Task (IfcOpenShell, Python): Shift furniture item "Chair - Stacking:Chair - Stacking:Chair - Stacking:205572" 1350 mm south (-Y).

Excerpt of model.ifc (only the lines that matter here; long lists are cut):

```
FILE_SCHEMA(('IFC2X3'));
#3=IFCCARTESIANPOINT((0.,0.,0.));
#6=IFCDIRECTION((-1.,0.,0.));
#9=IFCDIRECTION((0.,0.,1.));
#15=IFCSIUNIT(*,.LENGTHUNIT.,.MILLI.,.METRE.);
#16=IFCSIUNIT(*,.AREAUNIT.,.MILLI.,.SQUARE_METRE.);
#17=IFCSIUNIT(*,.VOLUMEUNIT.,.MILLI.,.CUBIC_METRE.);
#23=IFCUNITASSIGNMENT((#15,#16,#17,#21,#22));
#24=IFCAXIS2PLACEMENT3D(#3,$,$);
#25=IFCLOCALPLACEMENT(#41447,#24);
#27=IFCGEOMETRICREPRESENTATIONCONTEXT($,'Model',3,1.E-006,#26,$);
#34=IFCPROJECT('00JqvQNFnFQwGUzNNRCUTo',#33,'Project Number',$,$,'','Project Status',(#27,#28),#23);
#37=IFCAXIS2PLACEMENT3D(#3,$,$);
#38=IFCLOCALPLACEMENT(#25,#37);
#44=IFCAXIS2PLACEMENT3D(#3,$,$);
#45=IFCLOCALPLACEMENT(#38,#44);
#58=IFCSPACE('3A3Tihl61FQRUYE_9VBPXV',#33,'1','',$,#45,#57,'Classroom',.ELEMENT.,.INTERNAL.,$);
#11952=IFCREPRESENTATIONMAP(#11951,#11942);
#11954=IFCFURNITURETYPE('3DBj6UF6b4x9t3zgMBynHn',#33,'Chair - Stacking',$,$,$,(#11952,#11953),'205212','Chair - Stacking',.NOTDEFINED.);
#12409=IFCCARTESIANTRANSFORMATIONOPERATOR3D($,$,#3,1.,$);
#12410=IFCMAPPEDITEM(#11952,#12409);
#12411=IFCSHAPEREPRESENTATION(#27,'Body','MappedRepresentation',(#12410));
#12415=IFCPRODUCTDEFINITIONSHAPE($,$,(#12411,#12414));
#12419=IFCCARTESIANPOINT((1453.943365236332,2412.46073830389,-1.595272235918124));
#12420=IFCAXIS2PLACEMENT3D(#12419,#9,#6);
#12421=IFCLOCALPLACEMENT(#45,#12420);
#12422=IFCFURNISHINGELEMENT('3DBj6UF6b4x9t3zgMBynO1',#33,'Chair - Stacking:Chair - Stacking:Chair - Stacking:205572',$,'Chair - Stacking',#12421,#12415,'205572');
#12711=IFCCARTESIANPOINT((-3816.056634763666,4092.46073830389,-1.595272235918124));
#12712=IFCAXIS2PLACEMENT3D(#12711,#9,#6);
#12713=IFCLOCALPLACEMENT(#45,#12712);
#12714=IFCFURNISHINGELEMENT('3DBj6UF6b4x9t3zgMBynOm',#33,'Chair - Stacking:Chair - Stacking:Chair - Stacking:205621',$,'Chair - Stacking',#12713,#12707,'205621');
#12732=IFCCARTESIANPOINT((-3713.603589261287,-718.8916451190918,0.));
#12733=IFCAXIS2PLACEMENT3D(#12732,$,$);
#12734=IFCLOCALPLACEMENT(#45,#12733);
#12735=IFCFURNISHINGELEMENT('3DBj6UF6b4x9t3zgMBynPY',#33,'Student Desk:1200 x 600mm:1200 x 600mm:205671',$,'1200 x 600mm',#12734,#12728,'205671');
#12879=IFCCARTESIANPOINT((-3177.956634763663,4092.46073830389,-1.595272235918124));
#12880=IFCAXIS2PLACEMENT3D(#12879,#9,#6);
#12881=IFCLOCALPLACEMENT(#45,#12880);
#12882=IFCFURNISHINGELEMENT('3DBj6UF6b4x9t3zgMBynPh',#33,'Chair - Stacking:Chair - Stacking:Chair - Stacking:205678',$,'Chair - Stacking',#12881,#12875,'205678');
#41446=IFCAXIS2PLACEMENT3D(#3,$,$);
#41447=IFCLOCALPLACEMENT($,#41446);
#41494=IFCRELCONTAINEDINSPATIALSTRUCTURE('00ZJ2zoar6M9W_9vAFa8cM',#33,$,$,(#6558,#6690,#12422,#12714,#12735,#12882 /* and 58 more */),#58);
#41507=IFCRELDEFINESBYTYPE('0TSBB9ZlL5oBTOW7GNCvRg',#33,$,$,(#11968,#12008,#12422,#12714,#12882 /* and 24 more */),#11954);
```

```python
import ifcopenshell
import ifcopenshell.api.geometry
import ifcopenshell.util.placement

model = ifcopenshell.open("model.ifc")

item = model.by_id(12422)
matrix = ifcopenshell.util.placement.get_local_placement(item.ObjectPlacement)
matrix[1, 3] -= 1350.0
ifcopenshell.api.geometry.edit_object_placement(model, product=item, matrix=matrix, is_si=False)

print(ifcopenshell.util.placement.get_local_placement(item.ObjectPlacement).round(3) + 0.0)

model.write("model_updated.ifc")
```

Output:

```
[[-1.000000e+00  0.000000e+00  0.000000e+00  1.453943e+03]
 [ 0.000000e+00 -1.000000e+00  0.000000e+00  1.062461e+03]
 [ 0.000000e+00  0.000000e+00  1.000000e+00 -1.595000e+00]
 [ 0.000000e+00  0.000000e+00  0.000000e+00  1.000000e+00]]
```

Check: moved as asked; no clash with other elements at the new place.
